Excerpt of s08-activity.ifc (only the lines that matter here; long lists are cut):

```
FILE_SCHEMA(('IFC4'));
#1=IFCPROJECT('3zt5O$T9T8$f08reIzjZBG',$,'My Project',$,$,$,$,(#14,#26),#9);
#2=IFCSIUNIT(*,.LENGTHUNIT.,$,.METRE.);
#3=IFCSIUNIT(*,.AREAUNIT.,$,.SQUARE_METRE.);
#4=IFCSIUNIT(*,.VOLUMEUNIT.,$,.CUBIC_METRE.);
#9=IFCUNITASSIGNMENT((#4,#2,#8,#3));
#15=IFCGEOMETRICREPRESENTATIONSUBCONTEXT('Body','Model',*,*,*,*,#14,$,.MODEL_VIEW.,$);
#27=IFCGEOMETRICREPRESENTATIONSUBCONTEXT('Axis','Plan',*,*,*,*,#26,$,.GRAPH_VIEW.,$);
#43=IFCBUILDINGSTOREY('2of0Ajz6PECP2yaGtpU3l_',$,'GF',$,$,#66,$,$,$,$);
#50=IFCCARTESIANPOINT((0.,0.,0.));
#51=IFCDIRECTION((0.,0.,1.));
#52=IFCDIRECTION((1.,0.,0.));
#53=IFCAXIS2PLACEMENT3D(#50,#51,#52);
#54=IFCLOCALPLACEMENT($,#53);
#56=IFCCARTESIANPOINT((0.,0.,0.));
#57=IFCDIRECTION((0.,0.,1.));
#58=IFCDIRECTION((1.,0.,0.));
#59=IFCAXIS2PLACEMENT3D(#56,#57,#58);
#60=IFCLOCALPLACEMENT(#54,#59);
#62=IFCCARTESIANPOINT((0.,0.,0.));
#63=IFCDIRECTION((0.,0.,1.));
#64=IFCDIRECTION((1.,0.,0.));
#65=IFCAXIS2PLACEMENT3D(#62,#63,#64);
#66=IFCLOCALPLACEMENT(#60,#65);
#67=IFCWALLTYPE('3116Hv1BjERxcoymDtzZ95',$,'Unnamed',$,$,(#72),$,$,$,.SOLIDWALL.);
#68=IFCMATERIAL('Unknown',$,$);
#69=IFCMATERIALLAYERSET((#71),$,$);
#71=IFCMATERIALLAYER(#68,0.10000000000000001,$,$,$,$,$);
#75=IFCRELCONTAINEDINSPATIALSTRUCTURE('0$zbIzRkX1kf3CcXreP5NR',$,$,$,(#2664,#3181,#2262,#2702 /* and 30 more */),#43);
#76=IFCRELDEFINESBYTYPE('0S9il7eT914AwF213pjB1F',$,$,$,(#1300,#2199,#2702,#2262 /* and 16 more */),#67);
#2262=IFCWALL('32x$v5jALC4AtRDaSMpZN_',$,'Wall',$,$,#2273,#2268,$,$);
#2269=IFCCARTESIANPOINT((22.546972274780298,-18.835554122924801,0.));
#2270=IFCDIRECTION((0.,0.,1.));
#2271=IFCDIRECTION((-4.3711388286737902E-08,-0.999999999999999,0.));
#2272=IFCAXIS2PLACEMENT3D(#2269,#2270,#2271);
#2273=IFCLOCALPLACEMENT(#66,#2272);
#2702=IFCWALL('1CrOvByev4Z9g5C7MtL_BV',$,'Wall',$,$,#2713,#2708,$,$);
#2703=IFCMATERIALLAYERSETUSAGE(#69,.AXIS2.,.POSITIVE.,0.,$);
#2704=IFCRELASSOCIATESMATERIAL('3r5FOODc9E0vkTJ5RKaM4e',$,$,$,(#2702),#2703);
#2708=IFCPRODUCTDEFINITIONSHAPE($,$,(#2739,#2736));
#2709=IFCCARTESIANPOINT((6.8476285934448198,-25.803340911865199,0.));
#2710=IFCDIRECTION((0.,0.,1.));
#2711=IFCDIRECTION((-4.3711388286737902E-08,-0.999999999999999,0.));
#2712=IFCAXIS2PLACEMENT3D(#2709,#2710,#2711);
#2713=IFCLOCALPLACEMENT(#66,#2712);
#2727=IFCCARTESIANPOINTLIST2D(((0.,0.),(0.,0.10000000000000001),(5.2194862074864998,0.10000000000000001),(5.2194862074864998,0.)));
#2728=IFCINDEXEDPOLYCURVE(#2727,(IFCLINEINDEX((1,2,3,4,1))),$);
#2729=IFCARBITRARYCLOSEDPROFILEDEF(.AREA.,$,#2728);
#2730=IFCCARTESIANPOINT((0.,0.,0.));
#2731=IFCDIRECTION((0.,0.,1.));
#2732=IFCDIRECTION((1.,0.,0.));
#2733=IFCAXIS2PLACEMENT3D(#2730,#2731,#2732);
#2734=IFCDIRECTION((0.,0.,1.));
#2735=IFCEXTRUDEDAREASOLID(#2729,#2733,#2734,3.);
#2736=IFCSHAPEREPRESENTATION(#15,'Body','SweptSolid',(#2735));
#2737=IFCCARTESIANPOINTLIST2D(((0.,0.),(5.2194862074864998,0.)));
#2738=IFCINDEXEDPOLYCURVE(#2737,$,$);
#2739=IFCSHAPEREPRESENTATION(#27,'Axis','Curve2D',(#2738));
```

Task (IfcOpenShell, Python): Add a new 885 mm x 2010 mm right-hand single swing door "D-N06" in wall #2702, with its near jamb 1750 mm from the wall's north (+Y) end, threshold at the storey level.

```python
import numpy as np
import ifcopenshell
import ifcopenshell.api.feature
import ifcopenshell.api.geometry
import ifcopenshell.api.root
import ifcopenshell.api.spatial
import ifcopenshell.geom
import ifcopenshell.util.element
import ifcopenshell.util.placement
import ifcopenshell.util.representation
import ifcopenshell.util.shape
import ifcopenshell.util.unit

model = ifcopenshell.open("s08-activity.ifc")
unit_scale = ifcopenshell.util.unit.calculate_unit_scale(model)
settings = ifcopenshell.geom.settings()


def volume(element):
    """Net volume in cubic metres, openings subtracted."""
    shape = ifcopenshell.geom.create_shape(settings, element)
    return ifcopenshell.util.shape.get_volume(shape.geometry)


wall = model.by_guid("1CrOvByev4Z9g5C7MtL_BV")
storey = ifcopenshell.util.element.get_container(wall, ifc_class="IfcBuildingStorey")
context = ifcopenshell.util.representation.get_context(model, "Model", "Body", "MODEL_VIEW")
before = volume(wall)

width, height, from_end, sill = 0.885, 2.01, 1.75, 0.0  # metres

# The wall runs along its own X axis, and the end named is its -X end.
wall_shape = ifcopenshell.geom.create_shape(settings, wall)
x, y, z = ifcopenshell.util.shape.get_vertices(wall_shape.geometry).T
start = x.min() + from_end
face, thickness = float(y.min()), float(y.max() - y.min())
wall_matrix = ifcopenshell.util.placement.get_local_placement(wall.ObjectPlacement)
level = ifcopenshell.util.placement.get_local_placement(storey.ObjectPlacement)[2, 3]


def in_wall(x, y):
    """Placement at x, y metres in the wall's axes, at sill height."""
    matrix = wall_matrix.copy()
    matrix[:, 3] = wall_matrix @ np.array([x / unit_scale, y / unit_scale, 0.0, 1.0])
    matrix[2, 3] = level + sill / unit_scale
    return matrix


# Opening: a box that overshoots both wall faces by 50 mm.
opening = ifcopenshell.api.root.create_entity(model, ifc_class="IfcOpeningElement", predefined_type="OPENING")
box = ifcopenshell.api.geometry.add_wall_representation(
    model, context=context, length=width, height=height, thickness=thickness + 0.1
)
ifcopenshell.api.geometry.assign_representation(model, product=opening, representation=box)
ifcopenshell.api.geometry.edit_object_placement(model, product=opening, matrix=in_wall(start, face - 0.05), is_si=False)
ifcopenshell.api.feature.add_feature(model, feature=opening, element=wall)

door = ifcopenshell.api.root.create_entity(model, ifc_class="IfcDoor", name="D-N06", predefined_type="DOOR")
door.OverallWidth, door.OverallHeight = width / unit_scale, height / unit_scale
door.OperationType = "SINGLE_SWING_RIGHT"
body = ifcopenshell.api.geometry.add_door_representation(
    model,
    context=context,
    overall_width=door.OverallWidth,
    overall_height=door.OverallHeight,
    operation_type="SINGLE_SWING_RIGHT",
    lining_properties={"LiningDepth": thickness / unit_scale, "ThresholdDepth": thickness / unit_scale},
)
ifcopenshell.api.geometry.assign_representation(model, product=door, representation=body)
ifcopenshell.api.spatial.assign_container(model, products=[door], relating_structure=storey)
ifcopenshell.api.feature.add_filling(model, opening=opening, element=door)

# The lining spans the wall, so the door starts at the wall face.
ifcopenshell.api.geometry.edit_object_placement(model, product=door, matrix=in_wall(start, face), is_si=False)

after = volume(wall)

print(f"wall volume {before:.3f} -> {after:.3f} m3")

model.write("s08-activity_edited.ifc")
```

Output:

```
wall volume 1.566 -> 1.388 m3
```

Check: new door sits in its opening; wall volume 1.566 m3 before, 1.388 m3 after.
